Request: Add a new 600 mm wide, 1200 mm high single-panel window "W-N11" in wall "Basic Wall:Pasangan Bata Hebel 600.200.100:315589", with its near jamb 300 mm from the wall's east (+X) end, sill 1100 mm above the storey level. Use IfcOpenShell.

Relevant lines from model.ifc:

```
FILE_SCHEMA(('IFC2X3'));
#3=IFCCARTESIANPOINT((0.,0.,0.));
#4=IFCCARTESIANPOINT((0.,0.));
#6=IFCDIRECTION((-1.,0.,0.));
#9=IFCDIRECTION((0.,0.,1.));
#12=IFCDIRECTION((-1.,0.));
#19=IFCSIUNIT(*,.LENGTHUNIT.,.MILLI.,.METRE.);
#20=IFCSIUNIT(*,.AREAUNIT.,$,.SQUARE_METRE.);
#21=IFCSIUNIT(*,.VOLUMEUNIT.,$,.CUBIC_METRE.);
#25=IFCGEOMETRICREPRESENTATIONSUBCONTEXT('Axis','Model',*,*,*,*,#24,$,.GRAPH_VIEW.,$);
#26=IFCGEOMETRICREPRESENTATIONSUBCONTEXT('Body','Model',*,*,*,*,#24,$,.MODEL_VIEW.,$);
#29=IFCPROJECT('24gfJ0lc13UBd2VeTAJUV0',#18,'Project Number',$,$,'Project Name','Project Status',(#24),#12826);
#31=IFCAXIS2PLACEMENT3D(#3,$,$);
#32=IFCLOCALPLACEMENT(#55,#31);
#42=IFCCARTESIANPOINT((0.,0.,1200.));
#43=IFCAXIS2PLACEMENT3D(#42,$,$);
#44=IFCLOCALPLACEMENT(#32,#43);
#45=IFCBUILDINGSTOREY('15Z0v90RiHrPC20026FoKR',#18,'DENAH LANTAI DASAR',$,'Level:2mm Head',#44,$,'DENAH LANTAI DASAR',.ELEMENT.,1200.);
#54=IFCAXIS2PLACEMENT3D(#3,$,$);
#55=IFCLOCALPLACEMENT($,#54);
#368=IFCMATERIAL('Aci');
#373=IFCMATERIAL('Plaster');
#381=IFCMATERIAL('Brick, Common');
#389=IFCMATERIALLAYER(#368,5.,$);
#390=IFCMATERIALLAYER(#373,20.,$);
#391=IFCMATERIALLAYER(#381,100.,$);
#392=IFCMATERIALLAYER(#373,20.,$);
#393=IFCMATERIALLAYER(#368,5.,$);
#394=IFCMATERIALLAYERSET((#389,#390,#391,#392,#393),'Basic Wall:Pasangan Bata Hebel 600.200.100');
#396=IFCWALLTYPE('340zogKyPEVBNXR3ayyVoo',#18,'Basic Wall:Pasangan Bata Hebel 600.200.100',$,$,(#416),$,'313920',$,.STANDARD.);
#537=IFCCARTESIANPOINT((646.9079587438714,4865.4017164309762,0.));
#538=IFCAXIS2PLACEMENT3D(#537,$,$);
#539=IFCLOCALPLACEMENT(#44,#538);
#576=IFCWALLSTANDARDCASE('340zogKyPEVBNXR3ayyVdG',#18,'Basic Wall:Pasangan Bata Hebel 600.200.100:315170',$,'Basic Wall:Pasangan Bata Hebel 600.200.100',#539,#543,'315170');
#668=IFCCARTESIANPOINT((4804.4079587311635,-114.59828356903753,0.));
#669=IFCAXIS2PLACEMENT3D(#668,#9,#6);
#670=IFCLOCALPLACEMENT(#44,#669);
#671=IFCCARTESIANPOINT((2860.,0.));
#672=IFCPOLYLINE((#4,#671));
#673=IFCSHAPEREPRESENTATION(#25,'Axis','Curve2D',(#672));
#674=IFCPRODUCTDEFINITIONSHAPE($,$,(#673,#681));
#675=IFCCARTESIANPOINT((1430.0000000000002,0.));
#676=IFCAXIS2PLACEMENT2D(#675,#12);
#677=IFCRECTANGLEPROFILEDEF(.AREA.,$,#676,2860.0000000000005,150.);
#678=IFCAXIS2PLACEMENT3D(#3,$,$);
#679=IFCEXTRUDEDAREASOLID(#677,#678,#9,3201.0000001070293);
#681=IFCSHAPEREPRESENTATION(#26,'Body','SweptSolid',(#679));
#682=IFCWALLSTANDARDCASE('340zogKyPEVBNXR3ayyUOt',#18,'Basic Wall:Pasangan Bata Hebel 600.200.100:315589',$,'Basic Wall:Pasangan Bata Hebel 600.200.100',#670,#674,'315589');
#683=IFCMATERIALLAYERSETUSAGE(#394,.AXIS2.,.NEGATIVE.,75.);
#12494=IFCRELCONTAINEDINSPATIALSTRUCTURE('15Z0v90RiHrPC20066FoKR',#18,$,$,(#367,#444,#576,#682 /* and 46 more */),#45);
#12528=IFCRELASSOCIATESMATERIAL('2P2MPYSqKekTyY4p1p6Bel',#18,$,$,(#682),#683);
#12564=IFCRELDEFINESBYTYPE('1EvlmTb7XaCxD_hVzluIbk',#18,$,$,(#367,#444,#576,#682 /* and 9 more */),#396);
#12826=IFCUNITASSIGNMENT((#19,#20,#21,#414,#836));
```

```python
import numpy as np
import ifcopenshell
import ifcopenshell.api.feature
import ifcopenshell.api.geometry
import ifcopenshell.api.root
import ifcopenshell.api.spatial
import ifcopenshell.api.type
import ifcopenshell.geom
import ifcopenshell.util.element
import ifcopenshell.util.placement
import ifcopenshell.util.representation
import ifcopenshell.util.shape
import ifcopenshell.util.unit

model = ifcopenshell.open("model.ifc")
unit_scale = ifcopenshell.util.unit.calculate_unit_scale(model)
settings = ifcopenshell.geom.settings()


def volume(element):
    """Net volume in cubic metres, openings subtracted."""
    shape = ifcopenshell.geom.create_shape(settings, element)
    return ifcopenshell.util.shape.get_volume(shape.geometry)


wall = model.by_guid("340zogKyPEVBNXR3ayyUOt")
storey = ifcopenshell.util.element.get_container(wall, ifc_class="IfcBuildingStorey")
context = ifcopenshell.util.representation.get_context(model, "Model", "Body", "MODEL_VIEW")
before = volume(wall)

width, height, from_end, sill = 0.6, 1.2, 0.3, 1.1  # metres

# The wall runs along its own X axis, and the end named is its -X end.
wall_shape = ifcopenshell.geom.create_shape(settings, wall)
x, y, z = ifcopenshell.util.shape.get_vertices(wall_shape.geometry).T
start = x.min() + from_end
face, thickness = float(y.min()), float(y.max() - y.min())
wall_matrix = ifcopenshell.util.placement.get_local_placement(wall.ObjectPlacement)
level = ifcopenshell.util.placement.get_local_placement(storey.ObjectPlacement)[2, 3]


def in_wall(x, y):
    """Placement at x, y metres in the wall's axes, at sill height."""
    matrix = wall_matrix.copy()
    matrix[:, 3] = wall_matrix @ np.array([x / unit_scale, y / unit_scale, 0.0, 1.0])
    matrix[2, 3] = level + sill / unit_scale
    return matrix


# Opening: a box that overshoots both wall faces by 50 mm.
opening = ifcopenshell.api.root.create_entity(model, ifc_class="IfcOpeningElement")
box = ifcopenshell.api.geometry.add_wall_representation(
    model, context=context, length=width, height=height, thickness=thickness + 0.1
)
ifcopenshell.api.geometry.assign_representation(model, product=opening, representation=box)
ifcopenshell.api.geometry.edit_object_placement(model, product=opening, matrix=in_wall(start, face - 0.05), is_si=False)
ifcopenshell.api.feature.add_feature(model, feature=opening, element=wall)

window = ifcopenshell.api.root.create_entity(model, ifc_class="IfcWindow", name="W-N11")
window.OverallWidth, window.OverallHeight = width / unit_scale, height / unit_scale
body = ifcopenshell.api.geometry.add_window_representation(
    model,
    context=context,
    overall_width=window.OverallWidth,
    overall_height=window.OverallHeight,
    partition_type="SINGLE_PANEL",
)
ifcopenshell.api.geometry.assign_representation(model, product=window, representation=body)
ifcopenshell.api.spatial.assign_container(model, products=[window], relating_structure=storey)
fills = ifcopenshell.api.feature.add_filling(model, opening=opening, element=window)
fills.OwnerHistory = window.OwnerHistory  # required in IFC2X3

# IFC2X3 keeps the operation on the window style.
style = ifcopenshell.api.root.create_entity(model, ifc_class="IfcWindowStyle", name="W-N11")
style.OperationType, style.ConstructionType = "SINGLE_PANEL", "NOTDEFINED"
style.ParameterTakesPrecedence = style.Sizeable = False
ifcopenshell.api.type.assign_type(model, related_objects=[window], relating_type=style)

# Centre the window in the wall's thickness.
ifcopenshell.api.geometry.edit_object_placement(model, product=window, matrix=in_wall(start, face), is_si=False)
window_shape = ifcopenshell.geom.create_shape(settings, window)
depth = ifcopenshell.util.shape.get_vertices(window_shape.geometry)[:, 1]
offset = face + thickness / 2 - (depth.min() + depth.max()) / 2
ifcopenshell.api.geometry.edit_object_placement(model, product=window, matrix=in_wall(start, offset), is_si=False)

after = volume(wall)

print(f"wall volume {before:.3f} -> {after:.3f} m3")

model.write("model_updated.ifc")
```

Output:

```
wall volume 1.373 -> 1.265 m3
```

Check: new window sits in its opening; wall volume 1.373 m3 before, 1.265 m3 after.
